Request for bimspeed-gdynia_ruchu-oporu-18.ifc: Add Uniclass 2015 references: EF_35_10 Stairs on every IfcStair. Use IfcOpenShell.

First a look at what the model holds.

```python
import ifcopenshell

model = ifcopenshell.open("bimspeed-gdynia_ruchu-oporu-18.ifc")
print(model.schema)
print("classifications:", [c.Name for c in model.by_type("IfcClassification")])
for ifc_class in ("IfcDoor", "IfcRoof", "IfcStair", "IfcWall", "IfcWindow"):
    print(ifc_class, len(model.by_type(ifc_class)))
```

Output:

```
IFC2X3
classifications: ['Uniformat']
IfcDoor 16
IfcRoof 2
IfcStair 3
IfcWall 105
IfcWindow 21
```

```python
import ifcopenshell
import ifcopenshell.api.classification

model = ifcopenshell.open("bimspeed-gdynia_ruchu-oporu-18.ifc")

# IFC2X3 requires Source and Edition and has no link from the project to the system.
system = model.create_entity("IfcClassification", Source="NBS", Edition="2015", Name="Uniclass 2015")

codes = {
    "IfcStair": ("EF_35_10", "Stairs"),
}
for ifc_class, (code, name) in codes.items():
    products = model.by_type(ifc_class)
    ifcopenshell.api.classification.add_reference(
        model, products=products, classification=system, identification=code, name=name
    )
    print(code, len(products))

model.write("bimspeed-gdynia_ruchu-oporu-18_updated.ifc")
```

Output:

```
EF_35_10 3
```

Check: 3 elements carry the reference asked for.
